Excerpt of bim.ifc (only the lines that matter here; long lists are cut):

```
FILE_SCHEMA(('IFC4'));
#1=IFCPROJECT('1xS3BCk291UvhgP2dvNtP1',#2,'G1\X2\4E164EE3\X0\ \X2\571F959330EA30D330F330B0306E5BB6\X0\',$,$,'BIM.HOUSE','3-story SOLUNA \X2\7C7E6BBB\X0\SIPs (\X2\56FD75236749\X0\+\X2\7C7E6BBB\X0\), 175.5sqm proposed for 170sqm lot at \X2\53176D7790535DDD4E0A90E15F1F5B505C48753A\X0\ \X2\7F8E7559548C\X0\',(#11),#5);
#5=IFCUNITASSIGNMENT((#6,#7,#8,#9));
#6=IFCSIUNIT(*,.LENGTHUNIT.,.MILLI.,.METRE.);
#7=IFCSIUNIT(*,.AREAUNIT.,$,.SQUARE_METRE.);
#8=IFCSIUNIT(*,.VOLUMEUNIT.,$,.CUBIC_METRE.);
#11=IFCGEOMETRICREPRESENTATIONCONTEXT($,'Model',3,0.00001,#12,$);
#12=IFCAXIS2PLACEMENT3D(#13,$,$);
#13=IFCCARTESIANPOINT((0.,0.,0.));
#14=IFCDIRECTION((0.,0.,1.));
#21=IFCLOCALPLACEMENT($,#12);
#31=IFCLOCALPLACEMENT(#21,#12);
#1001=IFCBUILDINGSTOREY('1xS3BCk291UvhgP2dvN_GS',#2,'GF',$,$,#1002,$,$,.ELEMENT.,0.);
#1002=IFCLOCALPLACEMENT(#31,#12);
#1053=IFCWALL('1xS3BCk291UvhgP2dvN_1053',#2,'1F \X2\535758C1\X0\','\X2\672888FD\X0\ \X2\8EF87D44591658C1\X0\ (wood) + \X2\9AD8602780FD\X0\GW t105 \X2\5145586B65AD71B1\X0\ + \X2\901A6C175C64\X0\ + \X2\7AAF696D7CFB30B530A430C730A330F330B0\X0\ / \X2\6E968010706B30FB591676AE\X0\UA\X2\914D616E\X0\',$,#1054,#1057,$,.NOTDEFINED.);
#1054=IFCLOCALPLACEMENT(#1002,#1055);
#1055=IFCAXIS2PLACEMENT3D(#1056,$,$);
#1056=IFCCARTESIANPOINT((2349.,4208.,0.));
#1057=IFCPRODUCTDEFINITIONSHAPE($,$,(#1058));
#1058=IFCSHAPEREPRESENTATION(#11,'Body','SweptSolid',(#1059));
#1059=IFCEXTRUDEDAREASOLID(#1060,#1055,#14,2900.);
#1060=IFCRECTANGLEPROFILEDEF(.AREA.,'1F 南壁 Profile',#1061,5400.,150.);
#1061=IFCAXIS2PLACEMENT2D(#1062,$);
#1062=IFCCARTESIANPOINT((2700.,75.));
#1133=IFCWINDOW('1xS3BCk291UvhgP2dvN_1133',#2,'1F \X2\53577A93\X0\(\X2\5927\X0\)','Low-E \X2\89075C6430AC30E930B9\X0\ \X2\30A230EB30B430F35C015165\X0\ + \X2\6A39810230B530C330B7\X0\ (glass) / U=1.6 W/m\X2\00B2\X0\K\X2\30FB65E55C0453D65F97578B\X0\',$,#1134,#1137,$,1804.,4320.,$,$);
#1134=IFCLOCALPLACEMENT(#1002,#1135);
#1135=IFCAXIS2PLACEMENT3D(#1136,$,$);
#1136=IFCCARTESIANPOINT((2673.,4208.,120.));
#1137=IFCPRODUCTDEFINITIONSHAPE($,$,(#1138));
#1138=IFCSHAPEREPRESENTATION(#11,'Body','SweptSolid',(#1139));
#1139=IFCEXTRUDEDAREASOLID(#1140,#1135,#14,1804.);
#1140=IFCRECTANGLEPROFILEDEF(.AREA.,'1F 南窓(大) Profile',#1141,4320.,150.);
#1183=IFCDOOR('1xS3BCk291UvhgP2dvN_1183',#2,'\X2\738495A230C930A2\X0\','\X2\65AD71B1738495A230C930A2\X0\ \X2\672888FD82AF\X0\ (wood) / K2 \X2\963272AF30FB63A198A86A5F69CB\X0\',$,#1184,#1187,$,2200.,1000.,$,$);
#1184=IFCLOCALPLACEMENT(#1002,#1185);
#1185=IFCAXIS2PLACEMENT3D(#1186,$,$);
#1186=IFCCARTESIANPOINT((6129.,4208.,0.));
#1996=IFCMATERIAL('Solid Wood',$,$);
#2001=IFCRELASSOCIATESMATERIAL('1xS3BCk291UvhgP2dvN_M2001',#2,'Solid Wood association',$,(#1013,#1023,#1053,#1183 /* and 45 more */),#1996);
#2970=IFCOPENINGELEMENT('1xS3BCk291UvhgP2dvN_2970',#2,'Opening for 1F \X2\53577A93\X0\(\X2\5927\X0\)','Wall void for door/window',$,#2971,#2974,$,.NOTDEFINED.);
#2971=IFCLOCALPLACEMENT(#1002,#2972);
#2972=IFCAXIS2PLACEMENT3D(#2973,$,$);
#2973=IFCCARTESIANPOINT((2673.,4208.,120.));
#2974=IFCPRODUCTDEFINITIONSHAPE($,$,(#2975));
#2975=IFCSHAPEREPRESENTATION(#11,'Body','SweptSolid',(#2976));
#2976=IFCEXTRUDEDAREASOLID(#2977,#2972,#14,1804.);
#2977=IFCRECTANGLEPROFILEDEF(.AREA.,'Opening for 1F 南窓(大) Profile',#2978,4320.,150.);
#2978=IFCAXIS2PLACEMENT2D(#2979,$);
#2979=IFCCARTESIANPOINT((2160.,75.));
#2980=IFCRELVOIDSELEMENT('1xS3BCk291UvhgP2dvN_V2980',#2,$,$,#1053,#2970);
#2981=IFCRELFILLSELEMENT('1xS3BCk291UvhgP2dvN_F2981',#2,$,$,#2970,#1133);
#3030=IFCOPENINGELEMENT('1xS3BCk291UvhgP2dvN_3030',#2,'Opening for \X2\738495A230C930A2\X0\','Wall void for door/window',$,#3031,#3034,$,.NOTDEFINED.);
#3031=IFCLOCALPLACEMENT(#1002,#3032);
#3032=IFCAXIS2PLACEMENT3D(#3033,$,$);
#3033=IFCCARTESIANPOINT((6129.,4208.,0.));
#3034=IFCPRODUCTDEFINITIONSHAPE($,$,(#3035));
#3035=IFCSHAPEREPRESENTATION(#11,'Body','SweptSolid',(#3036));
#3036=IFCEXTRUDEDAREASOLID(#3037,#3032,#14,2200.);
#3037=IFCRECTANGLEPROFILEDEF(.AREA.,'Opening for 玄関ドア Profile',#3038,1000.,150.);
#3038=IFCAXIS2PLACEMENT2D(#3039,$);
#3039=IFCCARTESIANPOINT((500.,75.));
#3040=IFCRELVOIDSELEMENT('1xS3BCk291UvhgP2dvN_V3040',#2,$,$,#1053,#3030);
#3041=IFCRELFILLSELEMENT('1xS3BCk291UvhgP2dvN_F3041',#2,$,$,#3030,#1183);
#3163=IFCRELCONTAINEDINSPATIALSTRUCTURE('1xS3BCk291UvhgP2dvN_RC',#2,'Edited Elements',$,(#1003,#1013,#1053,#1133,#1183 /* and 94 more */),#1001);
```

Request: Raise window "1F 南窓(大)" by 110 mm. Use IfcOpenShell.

```python
import numpy as np
import ifcopenshell
import ifcopenshell.api.geometry
import ifcopenshell.util.placement
import ifcopenshell.util.unit

model = ifcopenshell.open("bim.ifc")
unit_scale = ifcopenshell.util.unit.calculate_unit_scale(model)

window = model.by_guid("1xS3BCk291UvhgP2dvN_1133")
opening = window.FillsVoids[0].RelatingOpeningElement
dz = 0.11 / unit_scale

shift = np.array([0.0, 0.0, dz])
# The window is not placed relative to its opening, so move both.
for product in (opening, window):
    matrix = ifcopenshell.util.placement.get_local_placement(product.ObjectPlacement)
    matrix[:3, 3] += shift
    ifcopenshell.api.geometry.edit_object_placement(model, product=product, matrix=matrix, is_si=False)

print(f"moved by {dz * unit_scale:+.3f} m")

model.write("bim_updated.ifc")
```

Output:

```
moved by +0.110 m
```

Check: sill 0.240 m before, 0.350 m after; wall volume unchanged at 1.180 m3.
